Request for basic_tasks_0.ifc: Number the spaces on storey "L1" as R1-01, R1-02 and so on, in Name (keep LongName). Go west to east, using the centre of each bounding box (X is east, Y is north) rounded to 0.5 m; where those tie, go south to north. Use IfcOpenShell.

First a look at what the model holds.

```python
import ifcopenshell
import ifcopenshell.util.element
import ifcopenshell.util.placement

model = ifcopenshell.open("basic_tasks_0.ifc")
print(model.schema)
storey = next(s for s in model.by_type("IfcBuildingStorey") if s.Name == "L1")
spaces = [e for e in ifcopenshell.util.element.get_decomposition(storey) if e.is_a("IfcSpace")]
for e in sorted(spaces, key=lambda e: e.id()):
    origin = ifcopenshell.util.placement.get_local_placement(e.ObjectPlacement)[:3, 3]
    print(e.id(), e.Name, e.LongName, origin.round(2) + 0.0, sep=" | ")
```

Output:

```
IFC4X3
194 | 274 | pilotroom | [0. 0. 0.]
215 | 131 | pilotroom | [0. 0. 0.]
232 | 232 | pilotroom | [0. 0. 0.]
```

```python
import ifcopenshell
import ifcopenshell.geom
import ifcopenshell.util.element
import ifcopenshell.util.shape

model = ifcopenshell.open("basic_tasks_0.ifc")
settings = ifcopenshell.geom.settings()
settings.set("use-world-coords", True)


def centre(element):
    shape = ifcopenshell.geom.create_shape(settings, element)
    return ifcopenshell.util.shape.get_bbox_centroid(shape.geometry)


storey = next(s for s in model.by_type("IfcBuildingStorey") if s.Name == "L1")
spaces = [e for e in ifcopenshell.util.element.get_decomposition(storey) if e.is_a("IfcSpace")]

# Insertion points can sit at a corner or the storey origin, so sort by the geometry (in metres).
centres = {e: centre(e) for e in spaces}
spaces.sort(key=lambda e: (round(centres[e][0] / 0.5), centres[e][1]))

for i, e in enumerate(spaces, start=1):
    number = f"R1-{i:02d}"
    e.Name = number
    print(e.id(), number)

model.write("basic_tasks_0-out.ifc")
```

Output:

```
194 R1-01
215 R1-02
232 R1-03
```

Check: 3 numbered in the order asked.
